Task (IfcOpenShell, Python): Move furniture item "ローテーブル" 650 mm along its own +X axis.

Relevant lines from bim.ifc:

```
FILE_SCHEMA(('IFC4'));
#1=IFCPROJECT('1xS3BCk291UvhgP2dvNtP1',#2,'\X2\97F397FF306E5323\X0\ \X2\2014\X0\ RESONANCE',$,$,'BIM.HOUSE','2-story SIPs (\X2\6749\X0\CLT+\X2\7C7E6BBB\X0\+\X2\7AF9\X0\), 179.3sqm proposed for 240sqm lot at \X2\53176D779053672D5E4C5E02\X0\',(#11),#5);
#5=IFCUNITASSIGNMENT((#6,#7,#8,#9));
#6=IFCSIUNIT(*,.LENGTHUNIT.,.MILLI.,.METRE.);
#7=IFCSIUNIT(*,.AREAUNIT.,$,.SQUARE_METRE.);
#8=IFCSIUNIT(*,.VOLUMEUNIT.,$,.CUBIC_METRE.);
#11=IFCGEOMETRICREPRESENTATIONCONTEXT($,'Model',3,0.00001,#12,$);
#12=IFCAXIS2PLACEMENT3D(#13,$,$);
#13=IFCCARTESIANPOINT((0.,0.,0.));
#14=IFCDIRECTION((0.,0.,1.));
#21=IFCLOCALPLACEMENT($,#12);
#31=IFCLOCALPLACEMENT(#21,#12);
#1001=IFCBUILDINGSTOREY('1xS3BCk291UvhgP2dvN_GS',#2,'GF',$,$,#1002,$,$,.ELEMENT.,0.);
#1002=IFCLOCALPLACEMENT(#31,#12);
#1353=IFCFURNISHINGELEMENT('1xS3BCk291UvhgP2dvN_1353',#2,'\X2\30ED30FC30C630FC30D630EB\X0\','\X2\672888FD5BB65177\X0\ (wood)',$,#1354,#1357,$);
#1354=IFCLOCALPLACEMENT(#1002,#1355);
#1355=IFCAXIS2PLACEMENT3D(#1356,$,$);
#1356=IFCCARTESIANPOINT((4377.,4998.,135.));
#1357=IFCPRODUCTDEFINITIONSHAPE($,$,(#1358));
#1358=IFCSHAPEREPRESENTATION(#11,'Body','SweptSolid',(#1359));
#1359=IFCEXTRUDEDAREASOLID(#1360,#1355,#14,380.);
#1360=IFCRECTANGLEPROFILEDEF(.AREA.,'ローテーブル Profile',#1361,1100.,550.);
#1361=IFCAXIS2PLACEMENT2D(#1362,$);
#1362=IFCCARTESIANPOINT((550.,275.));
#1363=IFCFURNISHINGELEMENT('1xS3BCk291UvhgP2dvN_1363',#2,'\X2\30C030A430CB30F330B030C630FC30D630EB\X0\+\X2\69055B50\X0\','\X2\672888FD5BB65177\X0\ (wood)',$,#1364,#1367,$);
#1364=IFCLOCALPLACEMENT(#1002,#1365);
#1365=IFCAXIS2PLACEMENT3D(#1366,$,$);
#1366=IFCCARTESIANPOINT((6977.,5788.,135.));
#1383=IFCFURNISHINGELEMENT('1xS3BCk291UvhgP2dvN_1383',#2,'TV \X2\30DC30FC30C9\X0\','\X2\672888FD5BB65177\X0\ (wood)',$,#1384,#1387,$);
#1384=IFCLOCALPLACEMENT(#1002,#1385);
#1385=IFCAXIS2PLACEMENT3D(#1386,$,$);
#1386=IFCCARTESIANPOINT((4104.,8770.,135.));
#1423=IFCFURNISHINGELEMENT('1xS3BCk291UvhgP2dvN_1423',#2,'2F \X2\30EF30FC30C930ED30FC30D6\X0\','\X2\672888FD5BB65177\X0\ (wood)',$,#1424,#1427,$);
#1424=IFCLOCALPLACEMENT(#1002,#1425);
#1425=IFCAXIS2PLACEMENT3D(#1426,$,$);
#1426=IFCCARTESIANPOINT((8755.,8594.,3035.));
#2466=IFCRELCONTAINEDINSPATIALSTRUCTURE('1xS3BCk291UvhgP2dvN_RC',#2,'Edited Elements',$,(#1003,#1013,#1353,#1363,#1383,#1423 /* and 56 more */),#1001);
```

```python
import ifcopenshell
import ifcopenshell.api.geometry
import ifcopenshell.util.placement
import ifcopenshell.util.unit

model = ifcopenshell.open("bim.ifc")
unit_scale = ifcopenshell.util.unit.calculate_unit_scale(model)

item = model.by_guid("1xS3BCk291UvhgP2dvN_1353")
matrix = ifcopenshell.util.placement.get_local_placement(item.ObjectPlacement)
matrix[:3, 3] += matrix[:3, 0] * 0.65 / unit_scale
ifcopenshell.api.geometry.edit_object_placement(model, product=item, matrix=matrix, is_si=False)

print(ifcopenshell.util.placement.get_local_placement(item.ObjectPlacement).round(3) + 0.0)

model.write("bim_v2.ifc")
```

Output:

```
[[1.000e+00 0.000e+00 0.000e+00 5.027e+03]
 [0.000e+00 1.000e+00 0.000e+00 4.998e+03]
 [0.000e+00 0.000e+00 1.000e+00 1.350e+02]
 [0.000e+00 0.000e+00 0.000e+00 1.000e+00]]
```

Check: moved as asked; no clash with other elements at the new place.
